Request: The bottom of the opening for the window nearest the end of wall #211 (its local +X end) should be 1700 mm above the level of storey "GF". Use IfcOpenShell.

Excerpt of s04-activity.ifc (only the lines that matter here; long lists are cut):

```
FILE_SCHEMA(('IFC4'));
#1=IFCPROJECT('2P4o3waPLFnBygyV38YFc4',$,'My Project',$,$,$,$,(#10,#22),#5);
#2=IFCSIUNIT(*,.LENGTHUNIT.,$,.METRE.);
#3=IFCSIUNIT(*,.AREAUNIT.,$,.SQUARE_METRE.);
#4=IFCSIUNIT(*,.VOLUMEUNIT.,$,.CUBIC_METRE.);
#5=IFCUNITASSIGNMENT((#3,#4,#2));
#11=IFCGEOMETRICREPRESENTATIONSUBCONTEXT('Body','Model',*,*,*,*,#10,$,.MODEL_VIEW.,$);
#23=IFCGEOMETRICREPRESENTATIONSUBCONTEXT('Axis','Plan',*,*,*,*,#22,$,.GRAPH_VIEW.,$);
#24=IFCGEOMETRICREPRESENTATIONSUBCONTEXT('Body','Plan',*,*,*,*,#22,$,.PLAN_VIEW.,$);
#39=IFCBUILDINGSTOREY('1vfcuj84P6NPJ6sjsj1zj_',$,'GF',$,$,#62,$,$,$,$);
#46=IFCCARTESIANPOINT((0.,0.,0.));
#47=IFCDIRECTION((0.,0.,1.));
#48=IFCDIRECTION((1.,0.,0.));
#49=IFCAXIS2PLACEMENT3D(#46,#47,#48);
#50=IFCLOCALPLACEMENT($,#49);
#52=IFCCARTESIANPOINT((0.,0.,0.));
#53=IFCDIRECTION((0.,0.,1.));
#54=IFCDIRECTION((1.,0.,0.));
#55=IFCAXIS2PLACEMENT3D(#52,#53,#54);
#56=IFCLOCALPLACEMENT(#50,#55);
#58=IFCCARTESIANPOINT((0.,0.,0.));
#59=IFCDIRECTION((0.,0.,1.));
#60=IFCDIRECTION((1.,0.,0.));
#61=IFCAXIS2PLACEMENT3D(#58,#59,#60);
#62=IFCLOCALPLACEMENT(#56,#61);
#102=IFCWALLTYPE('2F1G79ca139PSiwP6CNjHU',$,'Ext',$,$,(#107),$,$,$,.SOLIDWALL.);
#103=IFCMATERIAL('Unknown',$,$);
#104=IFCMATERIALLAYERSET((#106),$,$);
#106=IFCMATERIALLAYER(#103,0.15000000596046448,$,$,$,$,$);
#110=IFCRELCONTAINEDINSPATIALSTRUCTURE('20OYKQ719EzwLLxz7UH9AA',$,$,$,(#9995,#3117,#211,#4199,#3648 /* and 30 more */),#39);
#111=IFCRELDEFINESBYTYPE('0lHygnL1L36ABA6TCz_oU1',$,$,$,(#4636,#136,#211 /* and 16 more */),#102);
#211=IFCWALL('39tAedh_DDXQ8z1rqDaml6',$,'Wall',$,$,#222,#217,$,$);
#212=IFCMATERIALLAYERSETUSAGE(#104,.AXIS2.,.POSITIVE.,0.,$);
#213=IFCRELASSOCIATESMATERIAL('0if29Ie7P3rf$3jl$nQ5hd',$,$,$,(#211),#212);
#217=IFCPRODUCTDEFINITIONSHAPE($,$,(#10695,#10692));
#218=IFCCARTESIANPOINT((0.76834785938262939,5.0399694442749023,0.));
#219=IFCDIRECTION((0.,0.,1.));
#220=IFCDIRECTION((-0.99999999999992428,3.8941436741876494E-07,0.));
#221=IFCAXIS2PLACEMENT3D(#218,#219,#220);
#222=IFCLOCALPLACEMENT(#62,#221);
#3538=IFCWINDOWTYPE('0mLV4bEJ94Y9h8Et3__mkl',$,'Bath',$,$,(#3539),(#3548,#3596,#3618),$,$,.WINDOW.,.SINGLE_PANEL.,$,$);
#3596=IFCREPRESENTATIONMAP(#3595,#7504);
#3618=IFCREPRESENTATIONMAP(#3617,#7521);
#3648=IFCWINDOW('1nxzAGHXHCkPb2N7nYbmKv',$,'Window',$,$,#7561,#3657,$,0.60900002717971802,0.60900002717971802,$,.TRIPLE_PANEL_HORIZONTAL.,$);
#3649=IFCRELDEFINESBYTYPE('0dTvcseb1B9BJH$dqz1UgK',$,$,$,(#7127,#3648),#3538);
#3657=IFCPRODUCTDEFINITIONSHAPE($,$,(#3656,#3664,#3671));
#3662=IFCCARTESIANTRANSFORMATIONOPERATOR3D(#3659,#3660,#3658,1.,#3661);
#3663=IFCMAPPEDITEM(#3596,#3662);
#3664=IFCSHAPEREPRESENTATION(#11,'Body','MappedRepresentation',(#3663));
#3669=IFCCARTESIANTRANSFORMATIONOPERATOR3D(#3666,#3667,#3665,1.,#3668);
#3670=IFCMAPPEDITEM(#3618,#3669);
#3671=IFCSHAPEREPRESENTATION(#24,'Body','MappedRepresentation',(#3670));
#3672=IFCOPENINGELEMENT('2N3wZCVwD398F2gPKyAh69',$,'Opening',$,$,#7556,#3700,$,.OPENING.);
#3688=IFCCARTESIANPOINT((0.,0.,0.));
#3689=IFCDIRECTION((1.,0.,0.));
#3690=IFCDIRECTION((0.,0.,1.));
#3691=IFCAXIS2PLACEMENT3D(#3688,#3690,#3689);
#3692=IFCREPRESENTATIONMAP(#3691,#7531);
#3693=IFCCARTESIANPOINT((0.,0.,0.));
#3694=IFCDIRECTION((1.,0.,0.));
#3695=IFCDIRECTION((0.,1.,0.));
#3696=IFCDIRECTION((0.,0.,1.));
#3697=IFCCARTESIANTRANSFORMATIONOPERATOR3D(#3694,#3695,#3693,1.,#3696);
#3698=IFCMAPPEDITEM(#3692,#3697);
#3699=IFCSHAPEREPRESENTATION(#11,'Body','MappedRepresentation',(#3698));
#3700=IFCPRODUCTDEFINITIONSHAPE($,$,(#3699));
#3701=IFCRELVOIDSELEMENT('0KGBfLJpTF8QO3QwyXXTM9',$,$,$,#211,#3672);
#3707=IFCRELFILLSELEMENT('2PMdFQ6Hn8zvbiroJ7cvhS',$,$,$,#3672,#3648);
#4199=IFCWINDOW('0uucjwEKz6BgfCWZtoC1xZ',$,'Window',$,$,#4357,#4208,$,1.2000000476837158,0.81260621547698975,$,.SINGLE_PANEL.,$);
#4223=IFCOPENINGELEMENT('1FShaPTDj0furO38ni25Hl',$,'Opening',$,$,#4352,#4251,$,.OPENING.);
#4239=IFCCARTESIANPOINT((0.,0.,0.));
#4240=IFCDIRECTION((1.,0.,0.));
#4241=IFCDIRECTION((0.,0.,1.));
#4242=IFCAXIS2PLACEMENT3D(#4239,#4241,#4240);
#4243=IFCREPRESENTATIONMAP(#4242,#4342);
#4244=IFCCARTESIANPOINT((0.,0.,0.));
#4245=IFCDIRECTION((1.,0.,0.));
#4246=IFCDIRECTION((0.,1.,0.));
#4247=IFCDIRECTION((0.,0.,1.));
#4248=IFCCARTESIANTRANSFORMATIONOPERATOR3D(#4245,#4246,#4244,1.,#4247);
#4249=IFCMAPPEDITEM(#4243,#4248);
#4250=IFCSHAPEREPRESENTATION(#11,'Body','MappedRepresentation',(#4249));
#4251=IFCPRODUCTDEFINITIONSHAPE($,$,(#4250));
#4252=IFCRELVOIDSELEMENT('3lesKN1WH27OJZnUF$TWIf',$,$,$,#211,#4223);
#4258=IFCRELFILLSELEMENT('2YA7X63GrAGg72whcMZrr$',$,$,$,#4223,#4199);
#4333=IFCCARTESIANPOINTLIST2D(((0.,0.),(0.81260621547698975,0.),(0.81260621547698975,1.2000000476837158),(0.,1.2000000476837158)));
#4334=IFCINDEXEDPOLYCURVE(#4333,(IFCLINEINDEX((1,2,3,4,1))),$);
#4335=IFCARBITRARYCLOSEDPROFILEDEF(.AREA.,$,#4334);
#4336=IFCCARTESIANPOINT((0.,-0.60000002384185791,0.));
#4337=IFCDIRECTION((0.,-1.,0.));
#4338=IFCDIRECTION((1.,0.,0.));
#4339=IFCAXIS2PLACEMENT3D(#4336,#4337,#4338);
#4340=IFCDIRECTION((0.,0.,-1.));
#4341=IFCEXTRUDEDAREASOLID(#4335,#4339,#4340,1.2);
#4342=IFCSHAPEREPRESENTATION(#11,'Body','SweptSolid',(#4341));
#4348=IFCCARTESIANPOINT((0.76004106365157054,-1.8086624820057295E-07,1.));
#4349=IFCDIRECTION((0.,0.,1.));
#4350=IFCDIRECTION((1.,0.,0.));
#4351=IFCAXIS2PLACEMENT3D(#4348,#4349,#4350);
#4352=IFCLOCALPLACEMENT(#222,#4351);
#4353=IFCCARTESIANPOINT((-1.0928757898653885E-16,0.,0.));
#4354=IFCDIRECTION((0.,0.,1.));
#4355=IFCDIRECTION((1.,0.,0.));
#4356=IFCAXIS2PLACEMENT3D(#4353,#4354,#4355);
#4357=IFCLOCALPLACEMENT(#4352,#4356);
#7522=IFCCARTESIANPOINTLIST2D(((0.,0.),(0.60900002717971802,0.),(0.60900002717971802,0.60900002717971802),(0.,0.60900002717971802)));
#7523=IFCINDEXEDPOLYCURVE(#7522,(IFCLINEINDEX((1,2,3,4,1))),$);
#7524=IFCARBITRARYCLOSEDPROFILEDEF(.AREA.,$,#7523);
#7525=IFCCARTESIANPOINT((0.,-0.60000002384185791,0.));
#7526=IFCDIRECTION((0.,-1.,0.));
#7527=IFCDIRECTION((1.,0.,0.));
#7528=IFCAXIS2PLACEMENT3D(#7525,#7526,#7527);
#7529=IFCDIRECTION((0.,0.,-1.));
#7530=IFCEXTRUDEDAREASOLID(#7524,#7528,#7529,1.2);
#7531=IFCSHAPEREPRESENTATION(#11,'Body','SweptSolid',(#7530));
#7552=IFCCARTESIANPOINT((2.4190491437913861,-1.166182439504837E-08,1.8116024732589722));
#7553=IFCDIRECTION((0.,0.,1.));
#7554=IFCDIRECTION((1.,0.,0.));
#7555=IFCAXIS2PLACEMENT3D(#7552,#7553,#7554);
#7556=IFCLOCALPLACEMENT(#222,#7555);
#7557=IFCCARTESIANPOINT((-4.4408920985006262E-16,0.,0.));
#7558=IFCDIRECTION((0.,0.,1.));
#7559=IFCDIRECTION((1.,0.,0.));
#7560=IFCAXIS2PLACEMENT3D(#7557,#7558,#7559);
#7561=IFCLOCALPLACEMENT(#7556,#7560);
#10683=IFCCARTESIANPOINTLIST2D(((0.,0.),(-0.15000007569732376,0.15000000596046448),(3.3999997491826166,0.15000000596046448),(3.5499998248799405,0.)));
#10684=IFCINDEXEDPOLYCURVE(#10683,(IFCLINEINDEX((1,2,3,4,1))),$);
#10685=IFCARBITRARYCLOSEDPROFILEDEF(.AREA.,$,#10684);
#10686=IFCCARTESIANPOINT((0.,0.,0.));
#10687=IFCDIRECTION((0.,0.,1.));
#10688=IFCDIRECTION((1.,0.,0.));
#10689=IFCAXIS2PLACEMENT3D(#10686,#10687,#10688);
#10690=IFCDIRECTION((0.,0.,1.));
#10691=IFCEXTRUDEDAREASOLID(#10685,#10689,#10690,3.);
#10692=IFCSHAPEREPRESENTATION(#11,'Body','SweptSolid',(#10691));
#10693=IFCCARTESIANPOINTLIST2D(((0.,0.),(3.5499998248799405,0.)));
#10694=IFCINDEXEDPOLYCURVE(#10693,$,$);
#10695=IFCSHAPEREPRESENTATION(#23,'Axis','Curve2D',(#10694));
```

```python
import numpy as np
import ifcopenshell
import ifcopenshell.api.geometry
import ifcopenshell.geom
import ifcopenshell.util.element
import ifcopenshell.util.placement
import ifcopenshell.util.shape
import ifcopenshell.util.unit

model = ifcopenshell.open("s04-activity.ifc")
unit_scale = ifcopenshell.util.unit.calculate_unit_scale(model)

window = model.by_guid("1nxzAGHXHCkPb2N7nYbmKv")
opening = window.FillsVoids[0].RelatingOpeningElement
storey = ifcopenshell.util.element.get_container(window, ifc_class="IfcBuildingStorey")
level = ifcopenshell.util.placement.get_local_placement(storey.ObjectPlacement)[2, 3]

# The opening's origin need not be at the sill, so measure its lowest point.
shape = ifcopenshell.geom.create_shape(ifcopenshell.geom.settings(), opening)
bottom = ifcopenshell.util.shape.get_shape_bottom_elevation(shape, shape.geometry) / unit_scale
dz = level + 1.7 / unit_scale - bottom

shift = np.array([0.0, 0.0, dz])
# The window is placed relative to its opening, so it follows when the opening moves.
matrix = ifcopenshell.util.placement.get_local_placement(opening.ObjectPlacement)
matrix[:3, 3] += shift
ifcopenshell.api.geometry.edit_object_placement(
    model, product=opening, matrix=matrix, is_si=False, should_transform_children=True
)

print(f"moved by {dz * unit_scale:+.3f} m")

model.write("s04-activity_updated.ifc")
```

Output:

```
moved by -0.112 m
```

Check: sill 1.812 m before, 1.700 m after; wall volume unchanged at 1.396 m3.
